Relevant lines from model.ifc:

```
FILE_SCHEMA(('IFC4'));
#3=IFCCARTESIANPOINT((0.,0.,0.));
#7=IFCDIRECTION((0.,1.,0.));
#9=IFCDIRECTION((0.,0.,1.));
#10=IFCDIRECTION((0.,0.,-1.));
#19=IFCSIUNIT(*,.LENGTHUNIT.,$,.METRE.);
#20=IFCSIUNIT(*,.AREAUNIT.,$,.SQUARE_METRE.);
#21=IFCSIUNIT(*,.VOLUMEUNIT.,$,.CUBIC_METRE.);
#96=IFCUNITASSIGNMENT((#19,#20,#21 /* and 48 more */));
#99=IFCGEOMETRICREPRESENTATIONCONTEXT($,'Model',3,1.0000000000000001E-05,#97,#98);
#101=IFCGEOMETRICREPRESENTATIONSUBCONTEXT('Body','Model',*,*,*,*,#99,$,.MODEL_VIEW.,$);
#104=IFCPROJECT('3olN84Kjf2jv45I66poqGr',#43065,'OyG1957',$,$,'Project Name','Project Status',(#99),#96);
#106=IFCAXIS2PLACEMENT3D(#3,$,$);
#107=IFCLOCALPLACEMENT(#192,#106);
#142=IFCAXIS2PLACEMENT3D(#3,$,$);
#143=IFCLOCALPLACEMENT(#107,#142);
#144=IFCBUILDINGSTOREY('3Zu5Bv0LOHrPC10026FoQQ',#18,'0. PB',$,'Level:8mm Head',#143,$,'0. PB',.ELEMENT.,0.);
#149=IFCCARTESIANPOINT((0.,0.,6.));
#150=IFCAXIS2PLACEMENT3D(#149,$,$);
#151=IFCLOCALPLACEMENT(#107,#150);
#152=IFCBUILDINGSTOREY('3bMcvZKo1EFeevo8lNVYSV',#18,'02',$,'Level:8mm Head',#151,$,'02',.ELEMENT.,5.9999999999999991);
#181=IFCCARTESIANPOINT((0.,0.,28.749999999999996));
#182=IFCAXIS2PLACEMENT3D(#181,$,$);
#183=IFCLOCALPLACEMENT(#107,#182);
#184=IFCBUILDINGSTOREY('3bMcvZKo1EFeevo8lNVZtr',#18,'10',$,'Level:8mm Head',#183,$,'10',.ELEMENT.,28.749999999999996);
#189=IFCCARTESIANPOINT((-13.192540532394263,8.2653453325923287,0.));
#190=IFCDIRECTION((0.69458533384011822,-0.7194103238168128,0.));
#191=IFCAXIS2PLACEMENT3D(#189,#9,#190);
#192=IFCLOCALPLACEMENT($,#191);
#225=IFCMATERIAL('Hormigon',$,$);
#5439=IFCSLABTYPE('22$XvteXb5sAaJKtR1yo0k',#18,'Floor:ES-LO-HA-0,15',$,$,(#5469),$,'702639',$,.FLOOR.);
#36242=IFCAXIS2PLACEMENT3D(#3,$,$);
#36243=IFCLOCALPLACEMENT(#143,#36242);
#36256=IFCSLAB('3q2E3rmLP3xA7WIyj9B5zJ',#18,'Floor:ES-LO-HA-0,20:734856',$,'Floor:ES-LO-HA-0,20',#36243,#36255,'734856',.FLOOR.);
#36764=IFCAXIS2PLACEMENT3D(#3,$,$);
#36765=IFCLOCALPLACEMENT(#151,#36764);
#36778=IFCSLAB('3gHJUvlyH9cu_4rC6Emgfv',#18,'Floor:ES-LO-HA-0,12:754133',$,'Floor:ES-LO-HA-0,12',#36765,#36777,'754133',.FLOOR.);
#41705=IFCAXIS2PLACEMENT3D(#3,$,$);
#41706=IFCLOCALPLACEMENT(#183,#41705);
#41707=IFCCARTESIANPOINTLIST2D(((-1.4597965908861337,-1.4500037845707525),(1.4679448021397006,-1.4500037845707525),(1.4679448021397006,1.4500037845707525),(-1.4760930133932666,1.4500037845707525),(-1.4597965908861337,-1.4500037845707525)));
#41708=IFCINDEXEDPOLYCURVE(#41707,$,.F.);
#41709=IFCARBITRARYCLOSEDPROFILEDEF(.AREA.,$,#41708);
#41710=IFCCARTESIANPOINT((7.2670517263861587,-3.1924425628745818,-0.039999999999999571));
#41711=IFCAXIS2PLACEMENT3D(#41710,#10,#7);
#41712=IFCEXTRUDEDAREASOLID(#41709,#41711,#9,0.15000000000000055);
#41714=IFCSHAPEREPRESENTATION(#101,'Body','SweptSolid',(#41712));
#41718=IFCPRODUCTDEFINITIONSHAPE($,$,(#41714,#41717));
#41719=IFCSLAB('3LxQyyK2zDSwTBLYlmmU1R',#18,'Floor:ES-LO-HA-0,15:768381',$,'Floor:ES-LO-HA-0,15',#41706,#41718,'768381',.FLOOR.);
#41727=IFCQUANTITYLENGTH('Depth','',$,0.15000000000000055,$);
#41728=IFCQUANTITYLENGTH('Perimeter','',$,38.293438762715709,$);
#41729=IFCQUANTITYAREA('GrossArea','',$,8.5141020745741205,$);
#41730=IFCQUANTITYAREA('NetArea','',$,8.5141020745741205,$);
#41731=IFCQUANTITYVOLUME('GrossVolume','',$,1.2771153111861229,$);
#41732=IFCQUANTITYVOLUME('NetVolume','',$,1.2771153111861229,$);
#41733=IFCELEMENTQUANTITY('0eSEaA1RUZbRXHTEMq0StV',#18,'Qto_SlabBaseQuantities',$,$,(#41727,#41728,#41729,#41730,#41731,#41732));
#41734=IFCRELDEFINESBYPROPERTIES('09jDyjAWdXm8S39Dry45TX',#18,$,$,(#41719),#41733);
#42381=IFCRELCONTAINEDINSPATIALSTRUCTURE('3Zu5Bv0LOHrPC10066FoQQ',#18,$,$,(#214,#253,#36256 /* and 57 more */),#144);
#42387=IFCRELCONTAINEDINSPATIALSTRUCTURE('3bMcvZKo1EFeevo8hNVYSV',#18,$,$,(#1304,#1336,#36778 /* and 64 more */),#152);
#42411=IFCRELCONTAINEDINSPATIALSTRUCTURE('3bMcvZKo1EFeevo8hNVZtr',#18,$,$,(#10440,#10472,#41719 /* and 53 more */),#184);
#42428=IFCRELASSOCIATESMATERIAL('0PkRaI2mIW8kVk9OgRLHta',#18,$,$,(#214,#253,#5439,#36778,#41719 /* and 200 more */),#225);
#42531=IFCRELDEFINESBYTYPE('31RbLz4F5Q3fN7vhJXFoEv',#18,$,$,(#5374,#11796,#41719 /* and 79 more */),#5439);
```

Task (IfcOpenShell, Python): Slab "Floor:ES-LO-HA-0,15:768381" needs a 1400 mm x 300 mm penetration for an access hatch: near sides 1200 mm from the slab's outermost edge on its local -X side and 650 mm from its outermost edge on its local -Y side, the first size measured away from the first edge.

```python
import numpy as np
import ifcopenshell
import ifcopenshell.api.feature
import ifcopenshell.api.geometry
import ifcopenshell.api.pset
import ifcopenshell.api.root
import ifcopenshell.geom
import ifcopenshell.util.element
import ifcopenshell.util.placement
import ifcopenshell.util.representation
import ifcopenshell.util.shape
import ifcopenshell.util.unit

model = ifcopenshell.open("model.ifc")
unit_scale = ifcopenshell.util.unit.calculate_unit_scale(model)
area_scale = ifcopenshell.util.unit.calculate_unit_scale(model, "AREAUNIT")
volume_scale = ifcopenshell.util.unit.calculate_unit_scale(model, "VOLUMEUNIT")
settings = ifcopenshell.geom.settings()


def volume(element):
    """Net volume in cubic metres, openings subtracted."""
    shape = ifcopenshell.geom.create_shape(settings, element)
    return ifcopenshell.util.shape.get_volume(shape.geometry)


slab = model.by_id(41719)
before = volume(slab)

# Extent in the slab's own axes, in metres. The edges named are its -X and -Y sides.
slab_shape = ifcopenshell.geom.create_shape(settings, slab)
vertices = ifcopenshell.util.shape.get_vertices(slab_shape.geometry)
x_min, y_min, bottom = vertices.min(axis=0)
top = vertices[:, 2].max()

opening = ifcopenshell.api.root.create_entity(model, ifc_class="IfcOpeningElement", name="Access hatch opening", predefined_type="OPENING")
context = ifcopenshell.util.representation.get_context(model, "Model", "Body", "MODEL_VIEW")
width, depth = 1.4, 0.3
outline = [(0.0, 0.0), (width, 0.0), (width, depth), (0.0, depth), (0.0, 0.0)]
# Overshoot both faces by 50 mm so the cut is clean.
shape = ifcopenshell.api.geometry.add_slab_representation(
    model, context=context, depth=top - bottom + 0.1, polyline=outline
)
ifcopenshell.api.geometry.assign_representation(model, product=opening, representation=shape)

matrix = ifcopenshell.util.placement.get_local_placement(slab.ObjectPlacement)
matrix[:, 3] = matrix @ np.append(np.array([x_min + 1.2, y_min + 0.65, bottom - 0.05]) / unit_scale, 1.0)
ifcopenshell.api.geometry.edit_object_placement(model, product=opening, matrix=matrix, is_si=False)
ifcopenshell.api.feature.add_feature(model, feature=opening, element=slab)

after = volume(slab)

# Update the slab's stored quantities.
qto = model.by_id(ifcopenshell.util.element.get_pset(slab, "Qto_SlabBaseQuantities", should_inherit=False)["id"])
ifcopenshell.api.pset.edit_qto(model, qto=qto, properties={
    "NetArea": after / (top - bottom) / area_scale,
    "NetVolume": after / volume_scale,
})

print(f"slab volume {before:.3f} -> {after:.3f} m3")

model.write("model-out.ifc")
```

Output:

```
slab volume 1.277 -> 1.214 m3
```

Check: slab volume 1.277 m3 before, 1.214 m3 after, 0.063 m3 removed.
